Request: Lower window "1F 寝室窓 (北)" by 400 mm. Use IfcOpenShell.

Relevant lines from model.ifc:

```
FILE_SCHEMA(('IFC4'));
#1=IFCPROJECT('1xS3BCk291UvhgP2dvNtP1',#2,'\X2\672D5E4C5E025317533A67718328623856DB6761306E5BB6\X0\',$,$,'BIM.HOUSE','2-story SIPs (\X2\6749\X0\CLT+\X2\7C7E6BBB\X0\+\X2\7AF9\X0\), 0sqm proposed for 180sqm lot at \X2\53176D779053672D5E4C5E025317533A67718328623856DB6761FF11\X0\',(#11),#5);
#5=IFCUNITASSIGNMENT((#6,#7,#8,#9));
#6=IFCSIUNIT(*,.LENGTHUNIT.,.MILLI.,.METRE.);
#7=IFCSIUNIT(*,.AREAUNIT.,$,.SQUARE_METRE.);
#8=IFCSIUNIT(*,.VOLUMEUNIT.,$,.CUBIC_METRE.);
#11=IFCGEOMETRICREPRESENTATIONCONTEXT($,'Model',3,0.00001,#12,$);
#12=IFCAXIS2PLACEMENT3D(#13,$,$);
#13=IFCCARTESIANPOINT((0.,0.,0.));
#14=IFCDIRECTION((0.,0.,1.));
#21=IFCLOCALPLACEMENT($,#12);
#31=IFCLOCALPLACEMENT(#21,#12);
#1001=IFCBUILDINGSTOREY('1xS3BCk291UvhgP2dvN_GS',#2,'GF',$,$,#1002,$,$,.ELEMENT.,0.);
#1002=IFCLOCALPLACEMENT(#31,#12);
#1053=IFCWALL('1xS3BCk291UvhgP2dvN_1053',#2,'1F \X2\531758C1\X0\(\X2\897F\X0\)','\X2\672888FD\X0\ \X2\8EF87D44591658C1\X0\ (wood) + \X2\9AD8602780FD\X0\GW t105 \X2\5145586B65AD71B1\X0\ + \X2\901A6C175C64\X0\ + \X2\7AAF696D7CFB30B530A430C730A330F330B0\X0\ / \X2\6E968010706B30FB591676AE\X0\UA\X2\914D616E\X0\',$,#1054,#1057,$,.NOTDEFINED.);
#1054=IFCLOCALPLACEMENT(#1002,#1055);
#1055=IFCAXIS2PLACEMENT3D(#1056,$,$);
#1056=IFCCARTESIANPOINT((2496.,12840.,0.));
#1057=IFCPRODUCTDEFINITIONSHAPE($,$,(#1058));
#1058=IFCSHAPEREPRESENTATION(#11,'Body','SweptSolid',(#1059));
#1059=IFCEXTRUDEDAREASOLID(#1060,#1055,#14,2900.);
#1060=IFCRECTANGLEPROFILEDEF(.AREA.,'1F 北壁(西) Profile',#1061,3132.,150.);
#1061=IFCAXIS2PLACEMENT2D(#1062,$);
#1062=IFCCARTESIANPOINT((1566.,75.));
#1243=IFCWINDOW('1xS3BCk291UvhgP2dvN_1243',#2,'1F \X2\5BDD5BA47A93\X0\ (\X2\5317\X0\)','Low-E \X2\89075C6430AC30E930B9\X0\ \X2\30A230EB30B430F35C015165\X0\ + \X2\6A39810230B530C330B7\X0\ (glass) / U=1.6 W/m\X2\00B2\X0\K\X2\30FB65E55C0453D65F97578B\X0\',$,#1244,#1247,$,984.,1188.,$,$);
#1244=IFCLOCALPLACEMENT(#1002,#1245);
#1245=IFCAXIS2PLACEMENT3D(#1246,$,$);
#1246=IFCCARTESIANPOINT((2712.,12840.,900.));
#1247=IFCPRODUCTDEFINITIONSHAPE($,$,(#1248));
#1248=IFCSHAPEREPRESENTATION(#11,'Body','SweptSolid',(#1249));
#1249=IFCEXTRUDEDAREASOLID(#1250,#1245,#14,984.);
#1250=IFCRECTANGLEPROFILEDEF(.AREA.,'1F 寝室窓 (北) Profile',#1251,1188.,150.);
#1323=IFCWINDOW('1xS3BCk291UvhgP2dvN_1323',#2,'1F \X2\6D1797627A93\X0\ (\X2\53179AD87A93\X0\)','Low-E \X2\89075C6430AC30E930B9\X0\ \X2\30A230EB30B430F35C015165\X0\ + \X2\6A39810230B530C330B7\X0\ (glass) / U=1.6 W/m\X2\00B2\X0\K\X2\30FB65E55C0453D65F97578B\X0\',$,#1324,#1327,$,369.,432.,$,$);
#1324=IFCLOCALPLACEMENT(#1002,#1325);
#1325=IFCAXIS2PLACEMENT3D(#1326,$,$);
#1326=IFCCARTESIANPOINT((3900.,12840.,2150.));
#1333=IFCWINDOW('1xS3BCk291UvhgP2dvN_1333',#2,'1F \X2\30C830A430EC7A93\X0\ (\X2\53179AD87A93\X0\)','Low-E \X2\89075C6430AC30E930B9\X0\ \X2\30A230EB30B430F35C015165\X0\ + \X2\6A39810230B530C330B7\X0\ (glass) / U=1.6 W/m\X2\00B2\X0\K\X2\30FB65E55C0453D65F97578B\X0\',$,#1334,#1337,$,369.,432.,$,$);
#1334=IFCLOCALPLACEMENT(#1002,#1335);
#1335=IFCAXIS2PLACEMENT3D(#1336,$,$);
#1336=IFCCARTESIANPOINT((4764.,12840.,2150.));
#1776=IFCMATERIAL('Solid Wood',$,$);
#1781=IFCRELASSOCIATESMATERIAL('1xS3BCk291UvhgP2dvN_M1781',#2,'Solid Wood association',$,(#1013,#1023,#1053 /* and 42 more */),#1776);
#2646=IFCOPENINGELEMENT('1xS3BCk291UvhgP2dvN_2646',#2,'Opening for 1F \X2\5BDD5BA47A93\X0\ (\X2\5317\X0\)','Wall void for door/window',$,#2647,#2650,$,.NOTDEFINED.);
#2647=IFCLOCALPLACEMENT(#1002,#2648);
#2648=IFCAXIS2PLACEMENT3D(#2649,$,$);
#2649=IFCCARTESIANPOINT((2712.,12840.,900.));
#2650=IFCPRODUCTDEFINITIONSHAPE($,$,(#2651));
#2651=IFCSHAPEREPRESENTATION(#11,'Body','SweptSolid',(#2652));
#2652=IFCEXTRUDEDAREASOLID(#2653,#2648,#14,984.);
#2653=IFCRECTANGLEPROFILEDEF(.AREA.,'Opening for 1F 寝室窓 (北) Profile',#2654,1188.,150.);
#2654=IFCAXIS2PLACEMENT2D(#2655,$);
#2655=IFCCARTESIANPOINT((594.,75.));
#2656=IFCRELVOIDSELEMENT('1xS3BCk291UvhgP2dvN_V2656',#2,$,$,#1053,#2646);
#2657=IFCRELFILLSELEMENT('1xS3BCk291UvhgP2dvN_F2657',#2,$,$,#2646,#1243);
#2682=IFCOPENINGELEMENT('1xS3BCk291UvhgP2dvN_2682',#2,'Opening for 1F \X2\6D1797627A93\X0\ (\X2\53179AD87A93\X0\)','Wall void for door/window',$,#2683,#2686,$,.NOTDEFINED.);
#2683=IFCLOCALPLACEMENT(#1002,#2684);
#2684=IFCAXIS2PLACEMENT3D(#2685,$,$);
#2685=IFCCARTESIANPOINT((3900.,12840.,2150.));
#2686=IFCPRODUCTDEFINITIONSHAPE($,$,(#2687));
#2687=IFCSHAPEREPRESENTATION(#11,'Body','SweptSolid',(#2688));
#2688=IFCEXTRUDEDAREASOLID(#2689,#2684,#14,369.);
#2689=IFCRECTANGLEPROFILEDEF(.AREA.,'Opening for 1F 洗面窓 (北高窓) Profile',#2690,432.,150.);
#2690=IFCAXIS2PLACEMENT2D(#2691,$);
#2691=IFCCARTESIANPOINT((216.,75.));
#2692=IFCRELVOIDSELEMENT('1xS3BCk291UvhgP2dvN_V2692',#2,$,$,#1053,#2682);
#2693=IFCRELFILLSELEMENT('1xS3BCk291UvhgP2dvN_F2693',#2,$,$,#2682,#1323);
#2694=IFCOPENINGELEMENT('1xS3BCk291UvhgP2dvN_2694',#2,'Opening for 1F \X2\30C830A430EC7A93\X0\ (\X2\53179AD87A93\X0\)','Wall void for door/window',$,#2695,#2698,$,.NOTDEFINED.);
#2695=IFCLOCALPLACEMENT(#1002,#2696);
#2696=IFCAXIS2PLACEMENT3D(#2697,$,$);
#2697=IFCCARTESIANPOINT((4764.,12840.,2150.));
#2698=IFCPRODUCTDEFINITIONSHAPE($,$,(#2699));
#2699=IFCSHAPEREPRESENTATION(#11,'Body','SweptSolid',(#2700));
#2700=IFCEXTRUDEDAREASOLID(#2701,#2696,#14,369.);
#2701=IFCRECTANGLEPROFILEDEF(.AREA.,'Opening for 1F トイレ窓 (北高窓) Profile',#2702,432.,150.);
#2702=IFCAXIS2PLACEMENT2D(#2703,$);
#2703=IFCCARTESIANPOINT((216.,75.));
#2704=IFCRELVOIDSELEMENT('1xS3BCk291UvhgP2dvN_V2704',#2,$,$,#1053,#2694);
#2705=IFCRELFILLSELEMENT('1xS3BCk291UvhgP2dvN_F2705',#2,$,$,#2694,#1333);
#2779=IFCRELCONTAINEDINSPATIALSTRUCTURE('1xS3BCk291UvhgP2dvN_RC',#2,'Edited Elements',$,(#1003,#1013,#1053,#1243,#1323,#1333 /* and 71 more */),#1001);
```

```python
import numpy as np
import ifcopenshell
import ifcopenshell.api.geometry
import ifcopenshell.util.placement
import ifcopenshell.util.unit

model = ifcopenshell.open("model.ifc")
unit_scale = ifcopenshell.util.unit.calculate_unit_scale(model)

window = model.by_guid("1xS3BCk291UvhgP2dvN_1243")
opening = window.FillsVoids[0].RelatingOpeningElement
dz = -0.4 / unit_scale

shift = np.array([0.0, 0.0, dz])
# The window is not placed relative to its opening, so move both.
for product in (opening, window):
    matrix = ifcopenshell.util.placement.get_local_placement(product.ObjectPlacement)
    matrix[:3, 3] += shift
    ifcopenshell.api.geometry.edit_object_placement(model, product=product, matrix=matrix, is_si=False)

print(f"moved by {dz * unit_scale:+.3f} m")

model.write("model_edited.ifc")
```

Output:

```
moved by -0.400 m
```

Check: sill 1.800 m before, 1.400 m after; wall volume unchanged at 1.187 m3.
